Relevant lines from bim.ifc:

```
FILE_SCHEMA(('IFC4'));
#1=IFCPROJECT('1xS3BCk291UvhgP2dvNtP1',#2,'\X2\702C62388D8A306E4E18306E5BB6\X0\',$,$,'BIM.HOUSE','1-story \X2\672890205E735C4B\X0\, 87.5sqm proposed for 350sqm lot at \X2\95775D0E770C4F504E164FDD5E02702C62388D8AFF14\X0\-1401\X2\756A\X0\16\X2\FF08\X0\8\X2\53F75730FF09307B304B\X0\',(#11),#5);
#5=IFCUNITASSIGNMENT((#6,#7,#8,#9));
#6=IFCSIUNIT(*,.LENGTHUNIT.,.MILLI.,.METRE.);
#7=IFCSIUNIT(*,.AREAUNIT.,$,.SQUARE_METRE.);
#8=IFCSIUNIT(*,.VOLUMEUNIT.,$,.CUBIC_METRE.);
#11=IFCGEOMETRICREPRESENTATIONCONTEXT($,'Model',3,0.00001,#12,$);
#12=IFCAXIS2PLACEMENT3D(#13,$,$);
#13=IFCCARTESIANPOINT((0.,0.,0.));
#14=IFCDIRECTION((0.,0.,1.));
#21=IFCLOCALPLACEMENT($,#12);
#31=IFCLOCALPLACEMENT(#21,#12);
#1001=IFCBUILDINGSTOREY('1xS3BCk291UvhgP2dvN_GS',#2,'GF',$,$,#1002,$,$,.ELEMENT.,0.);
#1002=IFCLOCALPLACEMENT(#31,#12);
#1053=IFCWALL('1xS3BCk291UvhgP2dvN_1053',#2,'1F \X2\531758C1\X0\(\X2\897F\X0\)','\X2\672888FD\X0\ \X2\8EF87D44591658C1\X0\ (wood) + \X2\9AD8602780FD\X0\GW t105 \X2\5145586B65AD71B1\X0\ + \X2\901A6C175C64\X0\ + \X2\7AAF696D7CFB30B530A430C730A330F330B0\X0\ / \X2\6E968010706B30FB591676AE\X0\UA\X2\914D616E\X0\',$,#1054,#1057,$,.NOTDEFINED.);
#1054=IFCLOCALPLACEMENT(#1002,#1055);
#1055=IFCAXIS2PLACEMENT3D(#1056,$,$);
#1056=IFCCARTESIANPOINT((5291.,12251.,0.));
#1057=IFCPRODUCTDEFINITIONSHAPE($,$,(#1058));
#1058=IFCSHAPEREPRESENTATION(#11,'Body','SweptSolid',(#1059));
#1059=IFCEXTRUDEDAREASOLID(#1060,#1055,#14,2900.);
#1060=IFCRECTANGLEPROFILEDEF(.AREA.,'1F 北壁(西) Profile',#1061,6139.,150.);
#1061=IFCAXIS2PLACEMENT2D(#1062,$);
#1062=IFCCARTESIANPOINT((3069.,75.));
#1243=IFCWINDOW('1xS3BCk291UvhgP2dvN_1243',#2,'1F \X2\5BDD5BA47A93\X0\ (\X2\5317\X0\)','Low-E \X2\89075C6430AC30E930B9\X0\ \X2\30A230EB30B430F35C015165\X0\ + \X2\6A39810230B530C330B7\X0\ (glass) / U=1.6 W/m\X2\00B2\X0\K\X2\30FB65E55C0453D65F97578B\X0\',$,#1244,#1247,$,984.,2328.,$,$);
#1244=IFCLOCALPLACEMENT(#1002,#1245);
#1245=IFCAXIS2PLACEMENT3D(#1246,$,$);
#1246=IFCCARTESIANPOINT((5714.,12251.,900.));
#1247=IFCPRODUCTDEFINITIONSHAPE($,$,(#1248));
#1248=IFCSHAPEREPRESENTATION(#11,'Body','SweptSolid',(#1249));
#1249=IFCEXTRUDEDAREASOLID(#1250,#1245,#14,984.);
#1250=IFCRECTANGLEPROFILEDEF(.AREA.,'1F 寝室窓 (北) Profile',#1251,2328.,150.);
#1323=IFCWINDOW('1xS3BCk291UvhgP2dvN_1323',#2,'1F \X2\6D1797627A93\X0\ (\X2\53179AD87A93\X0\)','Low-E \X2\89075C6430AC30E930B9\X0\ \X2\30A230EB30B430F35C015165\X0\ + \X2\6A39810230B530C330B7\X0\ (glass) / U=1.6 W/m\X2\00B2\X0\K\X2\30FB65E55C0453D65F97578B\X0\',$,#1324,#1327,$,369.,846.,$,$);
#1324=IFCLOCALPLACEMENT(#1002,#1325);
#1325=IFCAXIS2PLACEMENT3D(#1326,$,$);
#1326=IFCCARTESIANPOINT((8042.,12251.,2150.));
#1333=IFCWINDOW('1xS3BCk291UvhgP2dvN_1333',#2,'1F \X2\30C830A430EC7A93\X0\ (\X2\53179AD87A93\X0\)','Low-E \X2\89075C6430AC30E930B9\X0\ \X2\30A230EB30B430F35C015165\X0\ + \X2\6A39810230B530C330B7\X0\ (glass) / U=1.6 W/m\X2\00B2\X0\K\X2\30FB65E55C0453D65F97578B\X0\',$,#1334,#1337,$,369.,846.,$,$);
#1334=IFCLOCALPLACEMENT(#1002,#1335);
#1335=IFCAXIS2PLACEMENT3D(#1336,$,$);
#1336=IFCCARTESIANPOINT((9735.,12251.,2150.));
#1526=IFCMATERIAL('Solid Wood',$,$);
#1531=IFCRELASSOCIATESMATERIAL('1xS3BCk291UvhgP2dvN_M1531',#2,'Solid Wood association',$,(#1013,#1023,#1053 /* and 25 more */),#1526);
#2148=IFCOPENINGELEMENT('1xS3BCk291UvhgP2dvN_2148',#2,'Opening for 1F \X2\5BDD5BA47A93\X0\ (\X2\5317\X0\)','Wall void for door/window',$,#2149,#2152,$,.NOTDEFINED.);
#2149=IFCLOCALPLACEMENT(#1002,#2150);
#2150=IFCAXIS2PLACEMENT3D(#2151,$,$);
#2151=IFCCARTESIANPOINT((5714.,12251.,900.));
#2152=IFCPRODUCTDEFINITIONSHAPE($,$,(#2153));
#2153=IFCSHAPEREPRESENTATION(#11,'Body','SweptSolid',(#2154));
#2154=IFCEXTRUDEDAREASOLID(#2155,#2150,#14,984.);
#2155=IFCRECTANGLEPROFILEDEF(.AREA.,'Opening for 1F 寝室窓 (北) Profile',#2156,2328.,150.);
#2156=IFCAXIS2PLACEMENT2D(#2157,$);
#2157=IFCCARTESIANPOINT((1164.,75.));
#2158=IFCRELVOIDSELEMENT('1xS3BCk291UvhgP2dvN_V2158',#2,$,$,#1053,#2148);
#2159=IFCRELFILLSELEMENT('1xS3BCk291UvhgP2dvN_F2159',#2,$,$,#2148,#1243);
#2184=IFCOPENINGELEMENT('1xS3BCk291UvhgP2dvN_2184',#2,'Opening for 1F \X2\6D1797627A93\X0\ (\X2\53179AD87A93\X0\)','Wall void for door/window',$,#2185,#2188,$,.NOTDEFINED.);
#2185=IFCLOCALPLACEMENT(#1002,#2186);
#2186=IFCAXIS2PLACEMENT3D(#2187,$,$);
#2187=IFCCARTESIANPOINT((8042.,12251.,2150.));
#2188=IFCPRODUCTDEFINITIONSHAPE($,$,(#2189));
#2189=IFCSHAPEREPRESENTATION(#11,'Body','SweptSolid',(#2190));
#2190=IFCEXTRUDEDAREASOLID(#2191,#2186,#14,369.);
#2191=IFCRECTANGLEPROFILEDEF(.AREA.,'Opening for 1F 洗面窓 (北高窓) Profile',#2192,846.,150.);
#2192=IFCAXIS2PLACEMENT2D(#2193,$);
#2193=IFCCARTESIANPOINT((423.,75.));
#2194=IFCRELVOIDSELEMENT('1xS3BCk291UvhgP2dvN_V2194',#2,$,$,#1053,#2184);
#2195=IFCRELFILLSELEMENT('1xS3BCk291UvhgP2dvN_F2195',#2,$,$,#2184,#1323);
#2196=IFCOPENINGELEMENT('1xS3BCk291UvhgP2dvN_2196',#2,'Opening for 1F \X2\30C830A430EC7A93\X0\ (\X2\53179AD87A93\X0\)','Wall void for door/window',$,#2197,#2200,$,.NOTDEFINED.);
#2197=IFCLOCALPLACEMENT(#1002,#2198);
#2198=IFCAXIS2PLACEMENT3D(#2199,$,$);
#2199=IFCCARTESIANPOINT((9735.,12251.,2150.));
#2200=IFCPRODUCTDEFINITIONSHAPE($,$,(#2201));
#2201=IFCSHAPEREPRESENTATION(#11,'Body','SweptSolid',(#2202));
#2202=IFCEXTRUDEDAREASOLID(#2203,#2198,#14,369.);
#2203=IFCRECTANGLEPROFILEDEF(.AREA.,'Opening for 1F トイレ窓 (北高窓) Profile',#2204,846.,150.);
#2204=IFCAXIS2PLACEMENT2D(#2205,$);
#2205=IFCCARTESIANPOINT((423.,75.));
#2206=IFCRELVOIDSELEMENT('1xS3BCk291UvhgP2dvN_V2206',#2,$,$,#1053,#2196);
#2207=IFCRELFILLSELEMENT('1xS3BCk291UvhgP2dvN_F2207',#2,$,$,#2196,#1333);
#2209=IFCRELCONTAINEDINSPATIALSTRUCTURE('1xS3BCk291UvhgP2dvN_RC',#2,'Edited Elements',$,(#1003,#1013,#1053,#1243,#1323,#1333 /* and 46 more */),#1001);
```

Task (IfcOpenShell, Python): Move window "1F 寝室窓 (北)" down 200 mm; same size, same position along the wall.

```python
import numpy as np
import ifcopenshell
import ifcopenshell.api.geometry
import ifcopenshell.util.placement
import ifcopenshell.util.unit

model = ifcopenshell.open("bim.ifc")
unit_scale = ifcopenshell.util.unit.calculate_unit_scale(model)

window = model.by_id(1243)
opening = window.FillsVoids[0].RelatingOpeningElement
dz = -200.0

shift = np.array([0.0, 0.0, dz])
# The window is not placed relative to its opening, so move both.
for product in (opening, window):
    matrix = ifcopenshell.util.placement.get_local_placement(product.ObjectPlacement)
    matrix[:3, 3] += shift
    ifcopenshell.api.geometry.edit_object_placement(model, product=product, matrix=matrix, is_si=False)

print(f"moved by {dz * unit_scale:+.3f} m")

model.write("bim_v2.ifc")
```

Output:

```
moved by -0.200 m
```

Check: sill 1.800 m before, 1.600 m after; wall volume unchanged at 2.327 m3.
